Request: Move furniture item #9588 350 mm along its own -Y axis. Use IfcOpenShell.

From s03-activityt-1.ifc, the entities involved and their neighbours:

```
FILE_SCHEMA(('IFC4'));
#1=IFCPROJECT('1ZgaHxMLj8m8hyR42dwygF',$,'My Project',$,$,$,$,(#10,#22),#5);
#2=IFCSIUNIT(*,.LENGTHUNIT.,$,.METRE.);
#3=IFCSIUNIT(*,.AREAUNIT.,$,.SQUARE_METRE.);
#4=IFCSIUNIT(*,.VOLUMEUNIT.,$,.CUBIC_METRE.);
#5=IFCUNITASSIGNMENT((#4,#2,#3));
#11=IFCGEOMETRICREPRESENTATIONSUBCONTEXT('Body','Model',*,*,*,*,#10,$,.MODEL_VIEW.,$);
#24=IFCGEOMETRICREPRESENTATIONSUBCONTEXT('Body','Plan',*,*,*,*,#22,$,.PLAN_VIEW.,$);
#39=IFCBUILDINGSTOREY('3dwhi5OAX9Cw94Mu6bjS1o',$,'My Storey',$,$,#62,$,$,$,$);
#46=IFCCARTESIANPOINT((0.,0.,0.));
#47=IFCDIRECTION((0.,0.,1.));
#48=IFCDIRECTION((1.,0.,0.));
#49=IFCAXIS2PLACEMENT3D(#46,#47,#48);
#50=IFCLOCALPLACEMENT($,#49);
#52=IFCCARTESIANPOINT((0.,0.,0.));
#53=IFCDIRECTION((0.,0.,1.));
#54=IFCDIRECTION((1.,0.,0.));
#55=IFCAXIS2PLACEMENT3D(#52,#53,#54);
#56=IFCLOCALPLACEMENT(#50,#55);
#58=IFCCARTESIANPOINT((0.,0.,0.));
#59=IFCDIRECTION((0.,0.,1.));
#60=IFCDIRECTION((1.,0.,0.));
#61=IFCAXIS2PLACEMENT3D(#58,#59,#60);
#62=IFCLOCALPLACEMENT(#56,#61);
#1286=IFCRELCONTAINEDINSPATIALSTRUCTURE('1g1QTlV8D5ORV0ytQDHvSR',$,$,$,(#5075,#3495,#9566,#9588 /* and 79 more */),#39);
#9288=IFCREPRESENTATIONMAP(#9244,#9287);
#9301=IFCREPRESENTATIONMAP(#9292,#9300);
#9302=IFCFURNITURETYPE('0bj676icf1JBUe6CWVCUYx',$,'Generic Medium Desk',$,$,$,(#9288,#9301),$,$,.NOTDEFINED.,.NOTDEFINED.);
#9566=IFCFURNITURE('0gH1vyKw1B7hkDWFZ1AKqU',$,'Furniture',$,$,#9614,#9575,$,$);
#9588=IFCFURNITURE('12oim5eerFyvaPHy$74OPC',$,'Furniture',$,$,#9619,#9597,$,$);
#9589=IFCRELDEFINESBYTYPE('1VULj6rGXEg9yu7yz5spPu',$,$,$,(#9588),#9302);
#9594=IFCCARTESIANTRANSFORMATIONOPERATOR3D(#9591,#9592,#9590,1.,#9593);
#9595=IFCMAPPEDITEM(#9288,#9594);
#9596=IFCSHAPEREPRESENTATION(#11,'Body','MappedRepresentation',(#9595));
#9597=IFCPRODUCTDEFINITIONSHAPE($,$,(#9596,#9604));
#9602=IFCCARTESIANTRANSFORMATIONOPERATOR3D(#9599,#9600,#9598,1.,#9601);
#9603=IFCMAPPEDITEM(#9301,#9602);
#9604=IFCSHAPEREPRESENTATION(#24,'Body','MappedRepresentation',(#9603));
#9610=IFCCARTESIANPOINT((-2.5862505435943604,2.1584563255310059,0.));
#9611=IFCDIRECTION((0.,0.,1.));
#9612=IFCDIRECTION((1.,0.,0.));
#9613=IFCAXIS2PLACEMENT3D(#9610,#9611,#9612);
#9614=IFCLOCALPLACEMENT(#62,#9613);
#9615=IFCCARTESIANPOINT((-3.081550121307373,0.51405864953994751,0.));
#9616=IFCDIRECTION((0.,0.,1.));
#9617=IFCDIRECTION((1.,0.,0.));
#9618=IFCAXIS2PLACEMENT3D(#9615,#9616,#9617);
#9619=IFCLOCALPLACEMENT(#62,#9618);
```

```python
import ifcopenshell
import ifcopenshell.api.geometry
import ifcopenshell.util.placement
import ifcopenshell.util.unit

model = ifcopenshell.open("s03-activityt-1.ifc")
unit_scale = ifcopenshell.util.unit.calculate_unit_scale(model)

item = model.by_guid("12oim5eerFyvaPHy$74OPC")
matrix = ifcopenshell.util.placement.get_local_placement(item.ObjectPlacement)
matrix[:3, 3] -= matrix[:3, 1] * 0.35 / unit_scale
ifcopenshell.api.geometry.edit_object_placement(model, product=item, matrix=matrix, is_si=False)

print(ifcopenshell.util.placement.get_local_placement(item.ObjectPlacement).round(3) + 0.0)

model.write("s03-activityt-1-out.ifc")
```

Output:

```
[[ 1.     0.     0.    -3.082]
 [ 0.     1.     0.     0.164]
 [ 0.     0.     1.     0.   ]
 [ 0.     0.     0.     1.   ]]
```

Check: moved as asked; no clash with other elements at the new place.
